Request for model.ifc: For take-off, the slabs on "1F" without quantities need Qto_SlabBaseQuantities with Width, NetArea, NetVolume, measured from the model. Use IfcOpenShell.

First a look at what the model holds.

```python
import ifcopenshell
import ifcopenshell.util.element
import ifcopenshell.util.unit

model = ifcopenshell.open("model.ifc")
print(model.schema)
for unit_type in ("LENGTHUNIT", "AREAUNIT", "VOLUMEUNIT"):
    print(unit_type, ifcopenshell.util.unit.calculate_unit_scale(model, unit_type))
storey = next(s for s in model.by_type("IfcBuildingStorey") if s.Name == "1F")
slabs = [e for e in ifcopenshell.util.element.get_decomposition(storey) if e.is_a("IfcSlab")]
for e in sorted(slabs, key=lambda e: e.id()):
    print(e.id(), e.is_a(), e.Name, list(ifcopenshell.util.element.get_psets(e, qtos_only=True)), sep=" | ")
```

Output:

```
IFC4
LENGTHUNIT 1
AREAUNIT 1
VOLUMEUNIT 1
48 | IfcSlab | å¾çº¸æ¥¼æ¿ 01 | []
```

```python
import ifcopenshell
import ifcopenshell.api.pset
import ifcopenshell.geom
import ifcopenshell.util.element
import ifcopenshell.util.shape
import ifcopenshell.util.unit

model = ifcopenshell.open("model.ifc")
unit_scale = ifcopenshell.util.unit.calculate_unit_scale(model)
area_scale = ifcopenshell.util.unit.calculate_unit_scale(model, "AREAUNIT")
volume_scale = ifcopenshell.util.unit.calculate_unit_scale(model, "VOLUMEUNIT")
settings = ifcopenshell.geom.settings()

storey = next(s for s in model.by_type("IfcBuildingStorey") if s.Name == "1F")
slabs = [e for e in ifcopenshell.util.element.get_decomposition(storey) if e.is_a("IfcSlab")]

for e in sorted(slabs, key=lambda e: e.id()):
    if ifcopenshell.util.element.get_psets(e, qtos_only=True, should_inherit=False):
        continue
    # Geometry comes back in metres, in the element's own axes.
    shape = ifcopenshell.geom.create_shape(settings, e)
    values = {
        "Width": ifcopenshell.util.shape.get_z(shape.geometry) / unit_scale,
        "NetArea": ifcopenshell.util.shape.get_footprint_area(shape.geometry) / area_scale,
        "NetVolume": ifcopenshell.util.shape.get_volume(shape.geometry) / volume_scale,
    }
    qto = ifcopenshell.api.pset.add_qto(model, product=e, name="Qto_SlabBaseQuantities")
    ifcopenshell.api.pset.edit_qto(model, qto=qto, properties=values)
    print(e.id(), {k: round(v, 3) for k, v in values.items()})

model.write("model_v2.ifc")
```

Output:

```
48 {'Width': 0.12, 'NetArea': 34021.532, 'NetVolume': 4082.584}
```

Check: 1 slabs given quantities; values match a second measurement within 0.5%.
